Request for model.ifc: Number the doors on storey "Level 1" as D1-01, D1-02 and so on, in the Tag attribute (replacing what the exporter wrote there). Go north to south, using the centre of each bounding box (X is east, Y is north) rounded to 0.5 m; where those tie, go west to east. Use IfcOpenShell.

First a look at what the model holds.

```python
import ifcopenshell
import ifcopenshell.util.element
import ifcopenshell.util.placement

model = ifcopenshell.open("model.ifc")
print(model.schema)
storey = next(s for s in model.by_type("IfcBuildingStorey") if s.Name == "Level 1")
doors = [e for e in ifcopenshell.util.element.get_decomposition(storey) if e.is_a("IfcDoor")]
for e in sorted(doors, key=lambda e: e.id()):
    origin = ifcopenshell.util.placement.get_local_placement(e.ObjectPlacement)[:3, 3]
    print(e.id(), e.Tag, e.Name, origin.round(2) + 0.0, sep=" | ")
```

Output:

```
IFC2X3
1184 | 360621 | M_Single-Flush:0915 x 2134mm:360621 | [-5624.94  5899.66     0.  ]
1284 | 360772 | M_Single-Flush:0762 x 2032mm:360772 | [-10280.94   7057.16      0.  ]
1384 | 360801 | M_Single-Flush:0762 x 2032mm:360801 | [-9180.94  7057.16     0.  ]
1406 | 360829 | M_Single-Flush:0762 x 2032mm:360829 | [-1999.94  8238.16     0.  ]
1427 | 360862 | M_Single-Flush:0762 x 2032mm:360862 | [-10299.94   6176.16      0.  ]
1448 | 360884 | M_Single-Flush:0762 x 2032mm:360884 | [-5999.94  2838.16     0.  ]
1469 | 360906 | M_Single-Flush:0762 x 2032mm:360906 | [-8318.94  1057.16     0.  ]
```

```python
import ifcopenshell
import ifcopenshell.geom
import ifcopenshell.util.element
import ifcopenshell.util.shape

model = ifcopenshell.open("model.ifc")
settings = ifcopenshell.geom.settings()
settings.set("use-world-coords", True)


def centre(element):
    shape = ifcopenshell.geom.create_shape(settings, element)
    return ifcopenshell.util.shape.get_bbox_centroid(shape.geometry)


storey = next(s for s in model.by_type("IfcBuildingStorey") if s.Name == "Level 1")
doors = [e for e in ifcopenshell.util.element.get_decomposition(storey) if e.is_a("IfcDoor")]

# Insertion points can sit at a corner or the storey origin, so sort by the geometry (in metres).
centres = {e: centre(e) for e in doors}
doors.sort(key=lambda e: (-round(centres[e][1] / 0.5), centres[e][0]))

for i, e in enumerate(doors, start=1):
    number = f"D1-{i:02d}"
    e.Tag = number
    print(e.id(), number)

model.write("model_updated.ifc")
```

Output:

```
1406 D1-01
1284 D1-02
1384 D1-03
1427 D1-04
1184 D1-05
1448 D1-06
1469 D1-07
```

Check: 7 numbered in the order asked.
